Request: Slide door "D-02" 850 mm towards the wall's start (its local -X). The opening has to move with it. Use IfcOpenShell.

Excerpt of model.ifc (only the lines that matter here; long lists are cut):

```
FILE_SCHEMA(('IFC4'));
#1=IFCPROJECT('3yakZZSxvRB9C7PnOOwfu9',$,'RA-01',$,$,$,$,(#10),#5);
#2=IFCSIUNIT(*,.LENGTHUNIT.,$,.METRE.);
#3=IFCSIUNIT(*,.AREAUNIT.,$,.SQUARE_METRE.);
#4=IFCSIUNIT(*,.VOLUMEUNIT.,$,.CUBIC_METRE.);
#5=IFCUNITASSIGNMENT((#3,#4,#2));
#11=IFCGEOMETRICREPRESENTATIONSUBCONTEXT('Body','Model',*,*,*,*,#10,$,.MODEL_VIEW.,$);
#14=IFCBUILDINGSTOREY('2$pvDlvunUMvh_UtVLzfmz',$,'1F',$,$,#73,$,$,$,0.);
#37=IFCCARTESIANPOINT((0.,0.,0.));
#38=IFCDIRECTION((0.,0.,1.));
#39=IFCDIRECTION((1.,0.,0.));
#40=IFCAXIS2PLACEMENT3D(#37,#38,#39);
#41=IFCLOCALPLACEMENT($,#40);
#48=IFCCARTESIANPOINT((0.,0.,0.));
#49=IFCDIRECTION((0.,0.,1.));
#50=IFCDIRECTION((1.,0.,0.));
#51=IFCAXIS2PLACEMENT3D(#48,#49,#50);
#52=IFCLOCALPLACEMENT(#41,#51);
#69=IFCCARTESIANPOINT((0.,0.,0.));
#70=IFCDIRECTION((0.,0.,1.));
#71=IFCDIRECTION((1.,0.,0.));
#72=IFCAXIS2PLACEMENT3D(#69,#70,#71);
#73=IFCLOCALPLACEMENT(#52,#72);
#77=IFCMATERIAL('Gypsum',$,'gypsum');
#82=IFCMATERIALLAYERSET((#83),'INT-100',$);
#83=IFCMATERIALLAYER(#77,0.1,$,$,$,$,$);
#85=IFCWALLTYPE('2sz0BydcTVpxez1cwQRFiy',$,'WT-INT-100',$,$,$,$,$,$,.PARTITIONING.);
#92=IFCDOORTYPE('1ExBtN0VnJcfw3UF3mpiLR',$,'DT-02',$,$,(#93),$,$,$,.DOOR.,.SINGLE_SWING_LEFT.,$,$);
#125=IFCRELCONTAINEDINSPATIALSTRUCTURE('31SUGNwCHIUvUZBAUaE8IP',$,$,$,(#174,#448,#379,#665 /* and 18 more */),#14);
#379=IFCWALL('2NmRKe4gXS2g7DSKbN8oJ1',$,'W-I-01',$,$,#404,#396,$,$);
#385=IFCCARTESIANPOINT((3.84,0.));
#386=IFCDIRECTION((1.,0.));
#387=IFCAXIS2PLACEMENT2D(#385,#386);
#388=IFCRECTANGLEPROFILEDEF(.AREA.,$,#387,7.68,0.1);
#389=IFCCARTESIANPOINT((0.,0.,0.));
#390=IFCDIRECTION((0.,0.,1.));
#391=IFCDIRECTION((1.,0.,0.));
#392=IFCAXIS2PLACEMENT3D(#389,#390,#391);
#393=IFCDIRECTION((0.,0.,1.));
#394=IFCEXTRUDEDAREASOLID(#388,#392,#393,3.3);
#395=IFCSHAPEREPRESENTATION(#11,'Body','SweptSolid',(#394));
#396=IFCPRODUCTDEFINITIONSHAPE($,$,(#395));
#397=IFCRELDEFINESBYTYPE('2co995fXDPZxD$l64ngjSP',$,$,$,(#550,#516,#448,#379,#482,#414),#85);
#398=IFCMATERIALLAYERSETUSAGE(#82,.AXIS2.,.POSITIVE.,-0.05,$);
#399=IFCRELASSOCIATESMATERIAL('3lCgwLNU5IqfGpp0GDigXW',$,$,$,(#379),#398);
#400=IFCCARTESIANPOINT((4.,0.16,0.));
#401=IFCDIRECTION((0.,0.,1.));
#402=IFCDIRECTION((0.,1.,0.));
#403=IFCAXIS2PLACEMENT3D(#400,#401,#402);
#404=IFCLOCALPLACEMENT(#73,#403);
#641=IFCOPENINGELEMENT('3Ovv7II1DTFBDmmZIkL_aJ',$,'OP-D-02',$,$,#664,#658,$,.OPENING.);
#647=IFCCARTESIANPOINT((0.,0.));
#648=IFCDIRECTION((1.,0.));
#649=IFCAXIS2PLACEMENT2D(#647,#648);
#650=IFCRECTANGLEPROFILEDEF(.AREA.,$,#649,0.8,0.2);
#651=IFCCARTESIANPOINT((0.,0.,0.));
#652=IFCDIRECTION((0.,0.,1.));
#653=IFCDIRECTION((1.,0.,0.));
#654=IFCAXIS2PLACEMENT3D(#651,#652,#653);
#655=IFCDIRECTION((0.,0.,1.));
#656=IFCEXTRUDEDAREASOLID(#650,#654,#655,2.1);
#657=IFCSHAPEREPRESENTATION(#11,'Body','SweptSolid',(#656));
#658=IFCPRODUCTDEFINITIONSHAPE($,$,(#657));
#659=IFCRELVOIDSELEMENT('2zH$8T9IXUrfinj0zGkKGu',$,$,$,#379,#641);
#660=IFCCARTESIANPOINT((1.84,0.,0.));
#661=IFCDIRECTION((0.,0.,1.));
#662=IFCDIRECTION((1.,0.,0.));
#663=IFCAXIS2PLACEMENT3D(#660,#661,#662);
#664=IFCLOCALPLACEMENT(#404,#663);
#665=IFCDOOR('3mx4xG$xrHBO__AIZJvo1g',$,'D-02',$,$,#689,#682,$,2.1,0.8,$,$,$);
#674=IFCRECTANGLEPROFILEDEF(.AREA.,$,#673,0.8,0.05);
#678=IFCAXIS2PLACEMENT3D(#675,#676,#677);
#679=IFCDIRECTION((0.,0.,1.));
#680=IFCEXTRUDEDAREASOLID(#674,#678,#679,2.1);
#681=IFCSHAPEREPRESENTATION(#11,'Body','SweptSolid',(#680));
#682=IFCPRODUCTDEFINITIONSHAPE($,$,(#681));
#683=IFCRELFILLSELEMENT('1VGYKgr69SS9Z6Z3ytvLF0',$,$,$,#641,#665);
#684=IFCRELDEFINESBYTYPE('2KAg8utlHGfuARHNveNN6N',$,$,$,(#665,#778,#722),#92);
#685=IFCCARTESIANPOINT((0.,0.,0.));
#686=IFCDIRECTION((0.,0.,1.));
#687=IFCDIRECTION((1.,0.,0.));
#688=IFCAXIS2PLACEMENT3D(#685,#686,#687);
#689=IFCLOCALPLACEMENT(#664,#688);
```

```python
import ifcopenshell
import ifcopenshell.api.geometry
import ifcopenshell.util.placement

model = ifcopenshell.open("model.ifc")

door = model.by_id(665)
opening = door.FillsVoids[0].RelatingOpeningElement
wall = opening.VoidsElements[0].RelatingBuildingElement

wall_matrix = ifcopenshell.util.placement.get_local_placement(wall.ObjectPlacement)
shift = wall_matrix[:3, 0] * -0.85
before = ifcopenshell.util.placement.get_local_placement(door.ObjectPlacement)[:3, 3].copy()

# The door is placed relative to its opening, so it follows when the opening moves.
matrix = ifcopenshell.util.placement.get_local_placement(opening.ObjectPlacement)
matrix[:3, 3] += shift
ifcopenshell.api.geometry.edit_object_placement(
    model, product=opening, matrix=matrix, is_si=False, should_transform_children=True
)

after = ifcopenshell.util.placement.get_local_placement(door.ObjectPlacement)[:3, 3]
print("door moved by", (after - before).round(3) + 0.0)

model.write("model_rev.ifc")
```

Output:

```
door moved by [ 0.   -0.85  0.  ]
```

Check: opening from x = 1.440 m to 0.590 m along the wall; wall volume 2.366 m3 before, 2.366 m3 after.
